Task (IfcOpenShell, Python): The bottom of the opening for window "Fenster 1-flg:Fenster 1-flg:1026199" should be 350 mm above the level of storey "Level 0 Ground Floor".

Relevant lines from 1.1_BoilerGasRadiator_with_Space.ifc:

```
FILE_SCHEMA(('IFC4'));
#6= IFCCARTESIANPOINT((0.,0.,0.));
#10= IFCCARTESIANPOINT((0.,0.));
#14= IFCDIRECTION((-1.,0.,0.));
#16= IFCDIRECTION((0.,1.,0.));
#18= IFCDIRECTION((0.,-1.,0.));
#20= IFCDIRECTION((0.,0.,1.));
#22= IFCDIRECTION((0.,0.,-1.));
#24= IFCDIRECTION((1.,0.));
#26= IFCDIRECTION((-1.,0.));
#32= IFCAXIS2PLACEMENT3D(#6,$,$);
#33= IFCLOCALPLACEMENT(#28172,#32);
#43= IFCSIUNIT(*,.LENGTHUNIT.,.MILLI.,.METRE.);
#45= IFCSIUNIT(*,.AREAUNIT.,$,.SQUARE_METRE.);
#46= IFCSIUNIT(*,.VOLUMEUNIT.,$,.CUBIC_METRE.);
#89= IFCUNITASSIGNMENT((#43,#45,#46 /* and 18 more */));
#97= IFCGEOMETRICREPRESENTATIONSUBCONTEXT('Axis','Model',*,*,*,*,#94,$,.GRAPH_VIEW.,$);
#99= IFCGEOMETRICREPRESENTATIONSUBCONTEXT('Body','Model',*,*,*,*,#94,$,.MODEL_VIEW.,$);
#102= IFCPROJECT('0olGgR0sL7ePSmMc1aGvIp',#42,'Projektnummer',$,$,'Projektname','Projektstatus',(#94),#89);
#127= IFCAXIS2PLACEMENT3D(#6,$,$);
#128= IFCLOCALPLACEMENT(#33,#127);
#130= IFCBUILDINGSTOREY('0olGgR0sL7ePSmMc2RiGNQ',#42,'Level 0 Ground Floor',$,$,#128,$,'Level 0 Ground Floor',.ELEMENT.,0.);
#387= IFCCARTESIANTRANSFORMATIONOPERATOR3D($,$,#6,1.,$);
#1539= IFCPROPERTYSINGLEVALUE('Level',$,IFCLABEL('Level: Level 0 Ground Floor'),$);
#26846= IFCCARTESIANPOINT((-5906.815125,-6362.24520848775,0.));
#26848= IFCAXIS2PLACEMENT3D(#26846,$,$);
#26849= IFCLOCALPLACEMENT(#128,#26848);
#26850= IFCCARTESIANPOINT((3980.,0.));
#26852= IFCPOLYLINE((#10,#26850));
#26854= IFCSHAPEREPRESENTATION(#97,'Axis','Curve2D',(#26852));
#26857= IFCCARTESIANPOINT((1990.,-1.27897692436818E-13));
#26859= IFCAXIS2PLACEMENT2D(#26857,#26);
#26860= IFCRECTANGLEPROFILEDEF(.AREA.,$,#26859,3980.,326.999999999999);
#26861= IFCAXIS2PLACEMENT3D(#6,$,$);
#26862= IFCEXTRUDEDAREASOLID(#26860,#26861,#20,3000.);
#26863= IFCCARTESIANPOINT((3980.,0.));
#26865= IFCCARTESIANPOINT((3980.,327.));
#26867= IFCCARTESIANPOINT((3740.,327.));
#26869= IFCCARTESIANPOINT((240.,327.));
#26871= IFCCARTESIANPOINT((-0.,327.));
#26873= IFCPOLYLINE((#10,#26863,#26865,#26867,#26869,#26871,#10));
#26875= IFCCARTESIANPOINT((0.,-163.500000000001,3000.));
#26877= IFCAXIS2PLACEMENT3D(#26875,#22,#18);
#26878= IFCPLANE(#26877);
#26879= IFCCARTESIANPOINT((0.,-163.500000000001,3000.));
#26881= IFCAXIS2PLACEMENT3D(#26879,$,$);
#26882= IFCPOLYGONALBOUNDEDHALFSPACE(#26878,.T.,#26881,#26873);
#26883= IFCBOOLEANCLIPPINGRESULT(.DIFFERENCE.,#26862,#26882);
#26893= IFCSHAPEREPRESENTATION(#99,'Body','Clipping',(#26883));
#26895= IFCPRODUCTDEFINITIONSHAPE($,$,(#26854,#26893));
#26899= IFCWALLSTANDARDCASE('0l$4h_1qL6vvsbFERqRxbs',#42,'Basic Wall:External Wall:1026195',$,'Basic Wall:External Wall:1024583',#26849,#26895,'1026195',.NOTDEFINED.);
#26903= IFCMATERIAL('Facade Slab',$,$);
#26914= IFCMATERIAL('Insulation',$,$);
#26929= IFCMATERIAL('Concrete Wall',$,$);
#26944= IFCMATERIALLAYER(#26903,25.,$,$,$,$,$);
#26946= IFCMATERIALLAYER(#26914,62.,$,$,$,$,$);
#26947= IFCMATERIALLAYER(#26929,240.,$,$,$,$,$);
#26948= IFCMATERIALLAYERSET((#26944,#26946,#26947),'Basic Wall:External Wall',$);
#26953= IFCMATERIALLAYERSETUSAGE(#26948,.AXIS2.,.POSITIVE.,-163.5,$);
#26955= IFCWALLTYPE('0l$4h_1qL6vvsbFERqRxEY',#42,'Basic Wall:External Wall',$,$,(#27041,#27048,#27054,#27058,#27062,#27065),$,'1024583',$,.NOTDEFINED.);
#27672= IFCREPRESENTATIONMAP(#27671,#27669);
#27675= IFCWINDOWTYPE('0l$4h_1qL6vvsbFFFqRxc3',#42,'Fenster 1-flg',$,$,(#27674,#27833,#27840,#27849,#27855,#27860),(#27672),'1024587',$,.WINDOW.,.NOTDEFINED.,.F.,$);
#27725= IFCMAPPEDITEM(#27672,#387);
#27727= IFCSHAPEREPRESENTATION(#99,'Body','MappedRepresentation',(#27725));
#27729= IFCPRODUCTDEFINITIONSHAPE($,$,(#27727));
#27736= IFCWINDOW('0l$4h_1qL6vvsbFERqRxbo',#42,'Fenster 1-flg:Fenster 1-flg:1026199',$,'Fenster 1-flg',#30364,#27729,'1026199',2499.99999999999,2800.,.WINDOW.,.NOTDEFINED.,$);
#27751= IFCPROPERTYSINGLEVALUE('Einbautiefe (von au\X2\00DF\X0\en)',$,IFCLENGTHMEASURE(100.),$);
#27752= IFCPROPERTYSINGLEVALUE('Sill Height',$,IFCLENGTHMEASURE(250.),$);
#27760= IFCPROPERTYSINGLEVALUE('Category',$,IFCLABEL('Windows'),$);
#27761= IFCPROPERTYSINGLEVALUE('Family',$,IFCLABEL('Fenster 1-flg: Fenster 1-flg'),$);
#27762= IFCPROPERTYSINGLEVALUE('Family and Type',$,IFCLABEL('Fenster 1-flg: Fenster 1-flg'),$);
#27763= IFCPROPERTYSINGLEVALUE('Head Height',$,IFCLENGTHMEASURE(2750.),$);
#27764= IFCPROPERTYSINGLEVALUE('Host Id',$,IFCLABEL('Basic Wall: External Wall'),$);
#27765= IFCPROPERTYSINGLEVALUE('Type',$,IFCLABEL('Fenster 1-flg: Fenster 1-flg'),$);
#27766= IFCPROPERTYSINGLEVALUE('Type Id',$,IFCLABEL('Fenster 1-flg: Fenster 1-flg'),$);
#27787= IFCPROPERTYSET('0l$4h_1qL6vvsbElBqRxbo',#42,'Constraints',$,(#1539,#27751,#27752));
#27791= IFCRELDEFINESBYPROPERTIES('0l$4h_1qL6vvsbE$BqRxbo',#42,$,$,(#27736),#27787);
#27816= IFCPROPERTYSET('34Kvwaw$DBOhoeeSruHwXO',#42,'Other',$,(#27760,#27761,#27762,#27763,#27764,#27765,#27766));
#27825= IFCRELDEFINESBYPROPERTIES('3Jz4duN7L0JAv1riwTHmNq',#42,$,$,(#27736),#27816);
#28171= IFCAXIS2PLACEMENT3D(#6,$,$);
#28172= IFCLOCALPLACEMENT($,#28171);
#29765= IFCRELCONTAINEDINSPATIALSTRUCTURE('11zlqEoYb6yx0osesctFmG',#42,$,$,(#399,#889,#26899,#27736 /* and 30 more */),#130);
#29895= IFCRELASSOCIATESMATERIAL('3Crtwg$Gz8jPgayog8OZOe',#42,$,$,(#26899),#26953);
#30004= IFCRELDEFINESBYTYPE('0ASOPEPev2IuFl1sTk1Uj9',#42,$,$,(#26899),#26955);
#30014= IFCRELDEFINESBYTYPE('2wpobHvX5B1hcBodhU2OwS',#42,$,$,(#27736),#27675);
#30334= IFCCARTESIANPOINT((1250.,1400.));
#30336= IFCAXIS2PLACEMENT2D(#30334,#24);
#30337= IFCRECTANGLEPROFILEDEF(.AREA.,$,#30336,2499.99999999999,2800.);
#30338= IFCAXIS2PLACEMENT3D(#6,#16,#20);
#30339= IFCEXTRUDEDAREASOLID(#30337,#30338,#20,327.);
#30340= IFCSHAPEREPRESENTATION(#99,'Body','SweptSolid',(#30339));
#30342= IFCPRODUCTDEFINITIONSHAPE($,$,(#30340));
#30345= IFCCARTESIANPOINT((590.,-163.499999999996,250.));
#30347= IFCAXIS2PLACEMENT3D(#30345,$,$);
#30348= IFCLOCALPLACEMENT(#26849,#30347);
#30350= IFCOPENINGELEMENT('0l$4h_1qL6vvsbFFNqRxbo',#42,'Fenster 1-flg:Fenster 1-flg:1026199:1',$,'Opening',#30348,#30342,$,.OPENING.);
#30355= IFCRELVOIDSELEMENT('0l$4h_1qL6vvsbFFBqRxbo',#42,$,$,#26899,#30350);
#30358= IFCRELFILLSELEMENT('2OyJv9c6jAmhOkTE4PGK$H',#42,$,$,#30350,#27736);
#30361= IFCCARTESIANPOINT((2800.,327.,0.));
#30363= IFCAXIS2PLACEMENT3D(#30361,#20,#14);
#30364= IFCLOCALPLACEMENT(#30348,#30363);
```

```python
import numpy as np
import ifcopenshell
import ifcopenshell.api.geometry
import ifcopenshell.api.pset
import ifcopenshell.geom
import ifcopenshell.util.element
import ifcopenshell.util.placement
import ifcopenshell.util.shape
import ifcopenshell.util.unit

model = ifcopenshell.open("1.1_BoilerGasRadiator_with_Space.ifc")
unit_scale = ifcopenshell.util.unit.calculate_unit_scale(model)

window = model.by_guid("0l$4h_1qL6vvsbFERqRxbo")
opening = window.FillsVoids[0].RelatingOpeningElement
storey = ifcopenshell.util.element.get_container(window, ifc_class="IfcBuildingStorey")
level = ifcopenshell.util.placement.get_local_placement(storey.ObjectPlacement)[2, 3]

# The opening's origin need not be at the sill, so measure its lowest point.
shape = ifcopenshell.geom.create_shape(ifcopenshell.geom.settings(), opening)
bottom = ifcopenshell.util.shape.get_shape_bottom_elevation(shape, shape.geometry) / unit_scale
dz = level + 0.35 / unit_scale - bottom

shift = np.array([0.0, 0.0, dz])
# The window is placed relative to its opening, so it follows when the opening moves.
matrix = ifcopenshell.util.placement.get_local_placement(opening.ObjectPlacement)
matrix[:3, 3] += shift
ifcopenshell.api.geometry.edit_object_placement(
    model, product=opening, matrix=matrix, is_si=False, should_transform_children=True
)

# Keep the stored heights in step.
pset = model.by_id(ifcopenshell.util.element.get_pset(window, "Constraints", should_inherit=False)["id"])
ifcopenshell.api.pset.edit_pset(model, pset=pset, properties={
    "Sill Height": model.create_entity("IfcLengthMeasure", ifcopenshell.util.element.get_pset(window, "Constraints", "Sill Height") + dz),
})
pset = model.by_id(ifcopenshell.util.element.get_pset(window, "Other", should_inherit=False)["id"])
ifcopenshell.api.pset.edit_pset(model, pset=pset, properties={
    "Head Height": model.create_entity("IfcLengthMeasure", ifcopenshell.util.element.get_pset(window, "Other", "Head Height") + dz),
})

print(f"moved by {dz * unit_scale:+.3f} m")

model.write("1.1_BoilerGasRadiator_with_Space_updated.ifc")
```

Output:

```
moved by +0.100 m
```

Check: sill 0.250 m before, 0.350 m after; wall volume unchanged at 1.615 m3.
